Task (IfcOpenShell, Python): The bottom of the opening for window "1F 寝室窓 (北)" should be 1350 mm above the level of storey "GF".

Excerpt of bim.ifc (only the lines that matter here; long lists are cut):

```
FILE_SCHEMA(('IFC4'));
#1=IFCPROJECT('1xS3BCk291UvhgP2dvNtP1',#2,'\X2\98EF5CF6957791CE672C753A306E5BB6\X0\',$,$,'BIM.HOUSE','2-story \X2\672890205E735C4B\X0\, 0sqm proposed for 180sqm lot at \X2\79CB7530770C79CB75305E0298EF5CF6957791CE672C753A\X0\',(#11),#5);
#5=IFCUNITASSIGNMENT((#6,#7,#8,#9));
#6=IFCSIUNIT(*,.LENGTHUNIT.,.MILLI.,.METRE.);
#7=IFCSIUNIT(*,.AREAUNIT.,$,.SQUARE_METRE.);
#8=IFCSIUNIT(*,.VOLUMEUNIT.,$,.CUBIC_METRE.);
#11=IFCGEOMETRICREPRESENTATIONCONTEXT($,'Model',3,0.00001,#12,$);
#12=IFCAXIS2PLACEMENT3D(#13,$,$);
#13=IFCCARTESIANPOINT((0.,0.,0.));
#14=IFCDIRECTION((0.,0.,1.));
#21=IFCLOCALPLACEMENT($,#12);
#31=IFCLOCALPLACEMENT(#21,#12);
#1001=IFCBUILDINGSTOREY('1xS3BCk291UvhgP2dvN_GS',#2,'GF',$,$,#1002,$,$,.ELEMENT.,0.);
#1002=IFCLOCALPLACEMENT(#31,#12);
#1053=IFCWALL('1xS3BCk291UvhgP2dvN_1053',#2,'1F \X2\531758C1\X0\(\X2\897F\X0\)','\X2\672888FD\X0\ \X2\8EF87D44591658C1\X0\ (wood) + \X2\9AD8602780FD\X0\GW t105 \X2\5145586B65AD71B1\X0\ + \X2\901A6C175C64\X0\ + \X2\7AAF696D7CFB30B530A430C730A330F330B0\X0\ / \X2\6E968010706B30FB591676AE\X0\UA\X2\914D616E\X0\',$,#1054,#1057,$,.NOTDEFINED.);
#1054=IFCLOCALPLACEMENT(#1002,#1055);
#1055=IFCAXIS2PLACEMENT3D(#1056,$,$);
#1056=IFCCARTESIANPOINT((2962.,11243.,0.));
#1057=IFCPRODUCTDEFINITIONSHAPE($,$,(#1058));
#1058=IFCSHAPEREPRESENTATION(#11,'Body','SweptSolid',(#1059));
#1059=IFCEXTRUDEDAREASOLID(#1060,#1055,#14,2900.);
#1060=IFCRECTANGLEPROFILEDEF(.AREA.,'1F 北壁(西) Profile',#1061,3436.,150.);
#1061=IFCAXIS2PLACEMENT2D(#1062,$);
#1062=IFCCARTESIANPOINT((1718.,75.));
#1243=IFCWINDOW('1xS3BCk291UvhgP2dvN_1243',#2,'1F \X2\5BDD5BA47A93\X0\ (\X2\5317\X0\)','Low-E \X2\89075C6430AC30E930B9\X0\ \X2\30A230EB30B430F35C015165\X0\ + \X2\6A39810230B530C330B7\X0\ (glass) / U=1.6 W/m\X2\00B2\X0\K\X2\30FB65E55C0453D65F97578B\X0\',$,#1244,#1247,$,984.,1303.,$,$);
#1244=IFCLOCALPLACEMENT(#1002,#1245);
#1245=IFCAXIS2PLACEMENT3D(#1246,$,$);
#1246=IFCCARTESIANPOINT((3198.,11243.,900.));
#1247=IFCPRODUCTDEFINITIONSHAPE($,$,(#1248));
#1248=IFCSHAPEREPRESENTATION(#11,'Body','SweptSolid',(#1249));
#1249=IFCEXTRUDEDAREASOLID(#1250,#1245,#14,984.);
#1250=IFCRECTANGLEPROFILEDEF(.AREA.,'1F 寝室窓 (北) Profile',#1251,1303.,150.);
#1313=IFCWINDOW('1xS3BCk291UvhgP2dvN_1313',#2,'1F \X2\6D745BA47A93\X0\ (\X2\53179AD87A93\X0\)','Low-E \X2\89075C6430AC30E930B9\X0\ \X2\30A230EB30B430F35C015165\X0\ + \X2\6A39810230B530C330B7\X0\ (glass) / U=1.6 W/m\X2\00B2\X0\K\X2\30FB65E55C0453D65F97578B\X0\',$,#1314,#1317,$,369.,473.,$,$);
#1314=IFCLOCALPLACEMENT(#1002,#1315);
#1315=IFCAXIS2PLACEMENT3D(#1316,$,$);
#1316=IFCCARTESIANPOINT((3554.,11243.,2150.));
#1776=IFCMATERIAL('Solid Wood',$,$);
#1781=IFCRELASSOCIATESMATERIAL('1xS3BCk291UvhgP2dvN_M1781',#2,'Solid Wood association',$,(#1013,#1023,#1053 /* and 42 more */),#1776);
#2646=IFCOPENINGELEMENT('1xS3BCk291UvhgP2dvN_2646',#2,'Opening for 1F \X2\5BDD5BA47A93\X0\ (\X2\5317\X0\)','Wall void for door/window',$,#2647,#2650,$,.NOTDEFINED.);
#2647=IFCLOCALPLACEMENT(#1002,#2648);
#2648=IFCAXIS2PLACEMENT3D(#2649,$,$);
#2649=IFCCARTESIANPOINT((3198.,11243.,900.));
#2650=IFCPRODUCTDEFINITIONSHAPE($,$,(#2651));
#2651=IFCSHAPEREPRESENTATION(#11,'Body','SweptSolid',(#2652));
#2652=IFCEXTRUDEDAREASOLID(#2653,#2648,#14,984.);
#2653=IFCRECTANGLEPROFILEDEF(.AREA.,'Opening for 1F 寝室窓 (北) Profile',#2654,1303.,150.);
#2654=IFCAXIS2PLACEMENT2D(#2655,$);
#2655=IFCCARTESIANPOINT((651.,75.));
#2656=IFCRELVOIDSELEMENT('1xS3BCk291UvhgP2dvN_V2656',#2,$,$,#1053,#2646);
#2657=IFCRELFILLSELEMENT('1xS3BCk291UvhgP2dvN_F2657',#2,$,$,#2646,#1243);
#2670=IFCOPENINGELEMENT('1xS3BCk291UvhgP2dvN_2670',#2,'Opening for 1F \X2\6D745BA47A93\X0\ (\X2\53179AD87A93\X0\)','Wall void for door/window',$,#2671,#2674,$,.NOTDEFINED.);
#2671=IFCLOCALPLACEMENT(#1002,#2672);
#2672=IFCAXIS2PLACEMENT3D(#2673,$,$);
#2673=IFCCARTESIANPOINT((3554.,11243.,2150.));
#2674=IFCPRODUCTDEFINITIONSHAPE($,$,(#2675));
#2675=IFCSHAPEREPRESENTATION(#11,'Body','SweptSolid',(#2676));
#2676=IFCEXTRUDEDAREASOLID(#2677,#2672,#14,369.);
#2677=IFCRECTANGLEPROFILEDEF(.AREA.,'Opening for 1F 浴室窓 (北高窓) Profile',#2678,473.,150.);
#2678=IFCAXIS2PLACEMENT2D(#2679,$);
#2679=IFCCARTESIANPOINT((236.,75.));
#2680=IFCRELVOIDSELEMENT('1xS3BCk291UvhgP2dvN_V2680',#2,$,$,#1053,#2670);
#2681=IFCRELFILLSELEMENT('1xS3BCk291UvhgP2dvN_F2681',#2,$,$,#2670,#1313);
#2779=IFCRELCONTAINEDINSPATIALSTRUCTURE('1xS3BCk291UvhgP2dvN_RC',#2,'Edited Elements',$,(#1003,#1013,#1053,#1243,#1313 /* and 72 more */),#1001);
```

```python
import numpy as np
import ifcopenshell
import ifcopenshell.api.geometry
import ifcopenshell.geom
import ifcopenshell.util.element
import ifcopenshell.util.placement
import ifcopenshell.util.shape
import ifcopenshell.util.unit

model = ifcopenshell.open("bim.ifc")
unit_scale = ifcopenshell.util.unit.calculate_unit_scale(model)

window = model.by_guid("1xS3BCk291UvhgP2dvN_1243")
opening = window.FillsVoids[0].RelatingOpeningElement
storey = ifcopenshell.util.element.get_container(window, ifc_class="IfcBuildingStorey")
level = ifcopenshell.util.placement.get_local_placement(storey.ObjectPlacement)[2, 3]

# The opening's origin need not be at the sill, so measure its lowest point.
shape = ifcopenshell.geom.create_shape(ifcopenshell.geom.settings(), opening)
bottom = ifcopenshell.util.shape.get_shape_bottom_elevation(shape, shape.geometry) / unit_scale
dz = level + 1.35 / unit_scale - bottom

shift = np.array([0.0, 0.0, dz])
# The window is not placed relative to its opening, so move both.
for product in (opening, window):
    matrix = ifcopenshell.util.placement.get_local_placement(product.ObjectPlacement)
    matrix[:3, 3] += shift
    ifcopenshell.api.geometry.edit_object_placement(model, product=product, matrix=matrix, is_si=False)

print(f"moved by {dz * unit_scale:+.3f} m")

model.write("bim-out.ifc")
```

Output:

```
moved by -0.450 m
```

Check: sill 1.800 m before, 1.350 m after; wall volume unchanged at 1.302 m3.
